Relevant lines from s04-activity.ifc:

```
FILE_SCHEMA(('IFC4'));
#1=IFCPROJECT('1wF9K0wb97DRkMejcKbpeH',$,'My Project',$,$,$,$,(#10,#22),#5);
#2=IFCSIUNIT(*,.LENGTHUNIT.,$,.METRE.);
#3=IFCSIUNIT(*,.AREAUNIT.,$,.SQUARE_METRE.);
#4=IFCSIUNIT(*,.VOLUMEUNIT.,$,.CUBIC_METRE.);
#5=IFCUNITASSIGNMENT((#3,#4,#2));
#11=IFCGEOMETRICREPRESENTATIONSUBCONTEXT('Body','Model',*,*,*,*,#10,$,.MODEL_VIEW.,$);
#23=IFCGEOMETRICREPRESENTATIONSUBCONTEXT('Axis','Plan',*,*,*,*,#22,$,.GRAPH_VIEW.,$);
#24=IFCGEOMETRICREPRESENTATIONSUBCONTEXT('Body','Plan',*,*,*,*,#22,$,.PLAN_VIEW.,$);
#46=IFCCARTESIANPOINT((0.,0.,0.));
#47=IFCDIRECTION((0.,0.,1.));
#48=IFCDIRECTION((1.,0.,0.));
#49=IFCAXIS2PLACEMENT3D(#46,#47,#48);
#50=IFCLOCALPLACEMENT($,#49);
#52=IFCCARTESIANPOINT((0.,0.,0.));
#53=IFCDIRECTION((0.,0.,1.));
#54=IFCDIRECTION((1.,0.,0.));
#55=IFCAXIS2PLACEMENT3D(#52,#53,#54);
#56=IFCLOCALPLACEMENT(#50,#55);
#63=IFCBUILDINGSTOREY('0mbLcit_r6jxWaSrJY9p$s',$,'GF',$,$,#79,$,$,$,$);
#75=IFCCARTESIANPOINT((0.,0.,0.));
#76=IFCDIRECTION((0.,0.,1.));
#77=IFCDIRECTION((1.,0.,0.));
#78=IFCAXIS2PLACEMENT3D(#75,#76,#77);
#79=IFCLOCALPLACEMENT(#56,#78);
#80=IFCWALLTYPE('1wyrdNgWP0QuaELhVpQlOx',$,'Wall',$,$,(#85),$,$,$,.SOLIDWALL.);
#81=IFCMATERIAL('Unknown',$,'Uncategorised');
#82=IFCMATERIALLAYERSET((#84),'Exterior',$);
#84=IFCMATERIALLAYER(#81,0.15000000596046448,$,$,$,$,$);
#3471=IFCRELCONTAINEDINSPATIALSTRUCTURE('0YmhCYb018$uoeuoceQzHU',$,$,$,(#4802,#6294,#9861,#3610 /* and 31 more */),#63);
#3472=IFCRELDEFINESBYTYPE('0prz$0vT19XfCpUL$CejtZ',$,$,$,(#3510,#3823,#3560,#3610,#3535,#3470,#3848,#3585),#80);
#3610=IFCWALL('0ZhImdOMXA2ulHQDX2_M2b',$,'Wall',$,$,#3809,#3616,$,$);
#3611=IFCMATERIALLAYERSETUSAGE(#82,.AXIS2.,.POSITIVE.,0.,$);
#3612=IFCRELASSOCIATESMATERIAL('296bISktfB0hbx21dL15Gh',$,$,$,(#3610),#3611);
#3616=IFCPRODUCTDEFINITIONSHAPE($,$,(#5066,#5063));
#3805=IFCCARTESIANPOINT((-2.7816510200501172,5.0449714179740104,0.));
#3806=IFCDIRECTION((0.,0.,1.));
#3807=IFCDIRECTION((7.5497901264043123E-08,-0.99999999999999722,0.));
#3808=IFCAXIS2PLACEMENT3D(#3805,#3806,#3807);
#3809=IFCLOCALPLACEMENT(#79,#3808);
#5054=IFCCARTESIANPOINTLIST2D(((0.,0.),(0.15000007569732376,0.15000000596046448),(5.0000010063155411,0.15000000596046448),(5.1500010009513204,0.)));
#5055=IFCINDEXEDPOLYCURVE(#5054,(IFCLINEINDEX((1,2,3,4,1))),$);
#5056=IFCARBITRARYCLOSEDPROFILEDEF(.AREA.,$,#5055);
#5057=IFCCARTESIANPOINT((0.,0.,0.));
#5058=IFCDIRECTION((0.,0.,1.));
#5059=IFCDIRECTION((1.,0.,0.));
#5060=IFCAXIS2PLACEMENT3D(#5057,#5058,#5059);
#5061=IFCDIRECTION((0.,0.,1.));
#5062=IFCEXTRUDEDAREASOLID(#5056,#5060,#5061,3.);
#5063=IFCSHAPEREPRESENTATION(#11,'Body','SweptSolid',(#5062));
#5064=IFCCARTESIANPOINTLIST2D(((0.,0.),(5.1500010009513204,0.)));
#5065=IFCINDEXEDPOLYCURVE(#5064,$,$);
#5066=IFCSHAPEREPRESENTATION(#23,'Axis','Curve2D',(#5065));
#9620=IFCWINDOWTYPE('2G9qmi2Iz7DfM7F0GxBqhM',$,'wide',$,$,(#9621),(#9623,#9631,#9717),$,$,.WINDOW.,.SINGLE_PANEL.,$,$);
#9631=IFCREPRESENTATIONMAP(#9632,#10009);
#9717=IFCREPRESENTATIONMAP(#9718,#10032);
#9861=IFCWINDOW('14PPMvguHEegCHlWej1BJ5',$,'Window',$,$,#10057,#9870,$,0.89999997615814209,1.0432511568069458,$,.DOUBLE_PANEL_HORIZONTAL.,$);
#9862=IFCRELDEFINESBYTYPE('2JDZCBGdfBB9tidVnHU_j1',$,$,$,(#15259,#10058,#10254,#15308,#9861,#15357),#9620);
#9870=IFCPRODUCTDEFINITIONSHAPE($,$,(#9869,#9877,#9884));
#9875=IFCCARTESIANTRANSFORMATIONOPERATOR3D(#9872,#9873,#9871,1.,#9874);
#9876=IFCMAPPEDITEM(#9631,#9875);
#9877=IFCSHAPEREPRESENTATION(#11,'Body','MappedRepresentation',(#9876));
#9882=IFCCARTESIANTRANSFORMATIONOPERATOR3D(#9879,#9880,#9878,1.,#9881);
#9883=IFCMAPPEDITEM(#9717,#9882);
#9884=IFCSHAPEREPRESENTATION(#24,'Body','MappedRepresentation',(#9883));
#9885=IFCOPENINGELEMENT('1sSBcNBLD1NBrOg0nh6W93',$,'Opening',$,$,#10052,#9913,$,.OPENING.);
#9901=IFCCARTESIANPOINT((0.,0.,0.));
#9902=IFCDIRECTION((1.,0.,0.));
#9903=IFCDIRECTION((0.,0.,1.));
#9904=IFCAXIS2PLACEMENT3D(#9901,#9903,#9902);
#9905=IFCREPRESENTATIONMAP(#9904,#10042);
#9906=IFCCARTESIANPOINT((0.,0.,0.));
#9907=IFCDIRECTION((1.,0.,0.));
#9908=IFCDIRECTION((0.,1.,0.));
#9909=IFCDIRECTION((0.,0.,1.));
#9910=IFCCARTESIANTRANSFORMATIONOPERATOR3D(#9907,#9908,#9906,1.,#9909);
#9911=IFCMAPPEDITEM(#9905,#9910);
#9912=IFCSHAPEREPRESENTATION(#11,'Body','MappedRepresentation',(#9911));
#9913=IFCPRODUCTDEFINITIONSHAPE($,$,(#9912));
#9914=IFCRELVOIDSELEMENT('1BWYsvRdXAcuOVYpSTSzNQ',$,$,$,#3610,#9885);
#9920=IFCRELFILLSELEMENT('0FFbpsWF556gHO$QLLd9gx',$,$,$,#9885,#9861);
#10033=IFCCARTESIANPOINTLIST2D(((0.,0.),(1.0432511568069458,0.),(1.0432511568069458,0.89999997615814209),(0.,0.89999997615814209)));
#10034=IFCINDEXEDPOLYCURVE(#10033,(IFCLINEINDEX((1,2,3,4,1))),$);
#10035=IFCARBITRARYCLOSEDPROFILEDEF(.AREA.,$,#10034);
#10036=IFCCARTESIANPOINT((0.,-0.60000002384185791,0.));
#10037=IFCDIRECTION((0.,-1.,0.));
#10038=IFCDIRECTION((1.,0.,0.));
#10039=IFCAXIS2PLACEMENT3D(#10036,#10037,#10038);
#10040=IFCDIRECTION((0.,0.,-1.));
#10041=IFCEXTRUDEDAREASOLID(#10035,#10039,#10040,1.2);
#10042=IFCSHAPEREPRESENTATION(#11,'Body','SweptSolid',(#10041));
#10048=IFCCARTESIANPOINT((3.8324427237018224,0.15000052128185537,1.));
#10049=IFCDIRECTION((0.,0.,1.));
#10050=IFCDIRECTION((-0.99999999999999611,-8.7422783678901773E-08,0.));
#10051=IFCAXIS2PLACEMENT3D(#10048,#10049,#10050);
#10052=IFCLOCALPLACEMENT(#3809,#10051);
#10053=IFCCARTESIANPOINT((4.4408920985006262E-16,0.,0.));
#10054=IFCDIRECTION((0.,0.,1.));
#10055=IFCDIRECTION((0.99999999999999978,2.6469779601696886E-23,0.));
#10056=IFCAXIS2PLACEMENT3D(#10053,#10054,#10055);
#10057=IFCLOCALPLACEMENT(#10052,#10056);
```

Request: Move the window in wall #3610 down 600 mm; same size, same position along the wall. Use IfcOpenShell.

```python
import numpy as np
import ifcopenshell
import ifcopenshell.api.geometry
import ifcopenshell.util.placement
import ifcopenshell.util.unit

model = ifcopenshell.open("s04-activity.ifc")
unit_scale = ifcopenshell.util.unit.calculate_unit_scale(model)

window = model.by_guid("14PPMvguHEegCHlWej1BJ5")
opening = window.FillsVoids[0].RelatingOpeningElement
dz = -0.6 / unit_scale

shift = np.array([0.0, 0.0, dz])
# The window is placed relative to its opening, so it follows when the opening moves.
matrix = ifcopenshell.util.placement.get_local_placement(opening.ObjectPlacement)
matrix[:3, 3] += shift
ifcopenshell.api.geometry.edit_object_placement(
    model, product=opening, matrix=matrix, is_si=False, should_transform_children=True
)

print(f"moved by {dz * unit_scale:+.3f} m")

model.write("s04-activity-out.ifc")
```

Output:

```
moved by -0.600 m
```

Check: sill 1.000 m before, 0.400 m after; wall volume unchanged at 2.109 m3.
